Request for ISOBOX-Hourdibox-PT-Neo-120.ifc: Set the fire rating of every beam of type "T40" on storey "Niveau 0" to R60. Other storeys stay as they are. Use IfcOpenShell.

First a look at what the model holds.

```python
import ifcopenshell
import ifcopenshell.util.element

model = ifcopenshell.open("ISOBOX-Hourdibox-PT-Neo-120.ifc")
print(model.schema)
storey = next(s for s in model.by_type("IfcBuildingStorey") if s.Name == "Niveau 0")
beams = [e for e in ifcopenshell.util.element.get_decomposition(storey) if e.is_a("IfcBeam")]
seen = {}
for e in beams:
    element_type = ifcopenshell.util.element.get_type(e)
    key = (element_type.Name if element_type != e and element_type else None, ifcopenshell.util.element.get_pset(e, "Pset_BeamCommon", "FireRating"))
    seen[key] = seen.get(key, 0) + 1
for (name, value), count in sorted(seen.items(), key=str):
    print(count, "x", name, "|", value)
```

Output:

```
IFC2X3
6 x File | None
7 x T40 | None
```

```python
import ifcopenshell
import ifcopenshell.api.pset
import ifcopenshell.util.element

model = ifcopenshell.open("ISOBOX-Hourdibox-PT-Neo-120.ifc")

storey = next(s for s in model.by_type("IfcBuildingStorey") if s.Name == "Niveau 0")
beams = [e for e in ifcopenshell.util.element.get_decomposition(storey) if e.is_a("IfcBeam")]

count = 0
for e in beams:
    element_type = ifcopenshell.util.element.get_type(e)
    if element_type in (None, e) or element_type.Name != "T40":
        continue
    # add_pset returns the element's existing set when there is one.
    pset = ifcopenshell.api.pset.add_pset(model, product=e, name="Pset_BeamCommon")
    ifcopenshell.api.pset.edit_pset(model, pset=pset, properties={"FireRating": "R60"})
    count += 1

print(count, "beams updated")

model.write("ISOBOX-Hourdibox-PT-Neo-120-out.ifc")
```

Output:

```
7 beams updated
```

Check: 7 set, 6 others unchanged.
